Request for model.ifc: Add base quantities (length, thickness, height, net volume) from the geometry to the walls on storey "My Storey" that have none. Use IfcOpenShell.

First a look at what the model holds.

```python
import ifcopenshell
import ifcopenshell.util.element
import ifcopenshell.util.unit

model = ifcopenshell.open("model.ifc")
print(model.schema)
for unit_type in ("LENGTHUNIT", "AREAUNIT", "VOLUMEUNIT"):
    print(unit_type, ifcopenshell.util.unit.calculate_unit_scale(model, unit_type))
storey = next(s for s in model.by_type("IfcBuildingStorey") if s.Name == "My Storey")
walls = [e for e in ifcopenshell.util.element.get_decomposition(storey) if e.is_a("IfcWall")]
for e in sorted(walls, key=lambda e: e.id()):
    print(e.id(), e.is_a(), e.Name, list(ifcopenshell.util.element.get_psets(e, qtos_only=True)), sep=" | ")
```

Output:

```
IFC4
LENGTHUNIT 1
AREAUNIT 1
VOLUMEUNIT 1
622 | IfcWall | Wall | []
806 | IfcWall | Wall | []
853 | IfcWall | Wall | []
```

```python
import ifcopenshell
import ifcopenshell.api.pset
import ifcopenshell.geom
import ifcopenshell.util.element
import ifcopenshell.util.shape
import ifcopenshell.util.unit

model = ifcopenshell.open("model.ifc")
unit_scale = ifcopenshell.util.unit.calculate_unit_scale(model)
volume_scale = ifcopenshell.util.unit.calculate_unit_scale(model, "VOLUMEUNIT")
settings = ifcopenshell.geom.settings()

storey = next(s for s in model.by_type("IfcBuildingStorey") if s.Name == "My Storey")
walls = [e for e in ifcopenshell.util.element.get_decomposition(storey) if e.is_a("IfcWall")]

for e in sorted(walls, key=lambda e: e.id()):
    if ifcopenshell.util.element.get_psets(e, qtos_only=True, should_inherit=False):
        continue
    # Geometry comes back in metres, in the element's own axes.
    shape = ifcopenshell.geom.create_shape(settings, e)
    values = {
        "Length": ifcopenshell.util.shape.get_x(shape.geometry) / unit_scale,
        "Width": ifcopenshell.util.shape.get_y(shape.geometry) / unit_scale,
        "Height": ifcopenshell.util.shape.get_z(shape.geometry) / unit_scale,
        "NetVolume": ifcopenshell.util.shape.get_volume(shape.geometry) / volume_scale,
    }
    qto = ifcopenshell.api.pset.add_qto(model, product=e, name="Qto_WallBaseQuantities")
    ifcopenshell.api.pset.edit_qto(model, qto=qto, properties=values)
    print(e.id(), {k: round(v, 3) for k, v in values.items()})

model.write("model-out.ifc")
```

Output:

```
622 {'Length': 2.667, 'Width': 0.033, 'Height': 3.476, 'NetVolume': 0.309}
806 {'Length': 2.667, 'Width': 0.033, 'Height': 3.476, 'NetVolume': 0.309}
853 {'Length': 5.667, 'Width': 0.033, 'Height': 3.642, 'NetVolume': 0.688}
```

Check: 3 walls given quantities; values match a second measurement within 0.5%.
